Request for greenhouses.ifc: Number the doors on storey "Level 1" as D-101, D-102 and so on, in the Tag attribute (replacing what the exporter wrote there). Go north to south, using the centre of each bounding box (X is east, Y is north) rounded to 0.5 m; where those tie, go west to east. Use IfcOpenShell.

First a look at what the model holds.

```python
import ifcopenshell
import ifcopenshell.util.element
import ifcopenshell.util.placement

model = ifcopenshell.open("greenhouses.ifc")
print(model.schema)
storey = next(s for s in model.by_type("IfcBuildingStorey") if s.Name == "Level 1")
doors = [e for e in ifcopenshell.util.element.get_decomposition(storey) if e.is_a("IfcDoor")]
for e in sorted(doors, key=lambda e: e.id()):
    origin = ifcopenshell.util.placement.get_local_placement(e.ObjectPlacement)[:3, 3]
    print(e.id(), e.Tag, e.Name, origin.round(2) + 0.0, sep=" | ")
```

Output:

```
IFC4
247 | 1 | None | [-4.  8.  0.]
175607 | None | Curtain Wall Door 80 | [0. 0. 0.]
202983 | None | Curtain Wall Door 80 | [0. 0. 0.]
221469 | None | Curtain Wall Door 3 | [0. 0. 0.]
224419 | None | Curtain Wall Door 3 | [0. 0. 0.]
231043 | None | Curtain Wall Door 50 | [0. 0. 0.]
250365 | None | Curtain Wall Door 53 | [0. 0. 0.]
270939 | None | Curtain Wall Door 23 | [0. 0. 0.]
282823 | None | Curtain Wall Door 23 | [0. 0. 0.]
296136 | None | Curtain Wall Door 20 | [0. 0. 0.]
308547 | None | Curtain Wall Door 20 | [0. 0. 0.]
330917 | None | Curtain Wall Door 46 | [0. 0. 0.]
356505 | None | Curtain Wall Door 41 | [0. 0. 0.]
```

```python
import ifcopenshell
import ifcopenshell.geom
import ifcopenshell.util.element
import ifcopenshell.util.shape

model = ifcopenshell.open("greenhouses.ifc")
settings = ifcopenshell.geom.settings()
settings.set("use-world-coords", True)


def centre(element):
    shape = ifcopenshell.geom.create_shape(settings, element)
    return ifcopenshell.util.shape.get_bbox_centroid(shape.geometry)


storey = next(s for s in model.by_type("IfcBuildingStorey") if s.Name == "Level 1")
doors = [e for e in ifcopenshell.util.element.get_decomposition(storey) if e.is_a("IfcDoor")]

# Insertion points can sit at a corner or the storey origin, so sort by the geometry (in metres).
centres = {e: centre(e) for e in doors}
doors.sort(key=lambda e: (-round(centres[e][1] / 0.5), centres[e][0]))

for i, e in enumerate(doors, start=1):
    number = f"D-1{i:02d}"
    e.Tag = number
    print(e.id(), number)

model.write("greenhouses_rev.ifc")
```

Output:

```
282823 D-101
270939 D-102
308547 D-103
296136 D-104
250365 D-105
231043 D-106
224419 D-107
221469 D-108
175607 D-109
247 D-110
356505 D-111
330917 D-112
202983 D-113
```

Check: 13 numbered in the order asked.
